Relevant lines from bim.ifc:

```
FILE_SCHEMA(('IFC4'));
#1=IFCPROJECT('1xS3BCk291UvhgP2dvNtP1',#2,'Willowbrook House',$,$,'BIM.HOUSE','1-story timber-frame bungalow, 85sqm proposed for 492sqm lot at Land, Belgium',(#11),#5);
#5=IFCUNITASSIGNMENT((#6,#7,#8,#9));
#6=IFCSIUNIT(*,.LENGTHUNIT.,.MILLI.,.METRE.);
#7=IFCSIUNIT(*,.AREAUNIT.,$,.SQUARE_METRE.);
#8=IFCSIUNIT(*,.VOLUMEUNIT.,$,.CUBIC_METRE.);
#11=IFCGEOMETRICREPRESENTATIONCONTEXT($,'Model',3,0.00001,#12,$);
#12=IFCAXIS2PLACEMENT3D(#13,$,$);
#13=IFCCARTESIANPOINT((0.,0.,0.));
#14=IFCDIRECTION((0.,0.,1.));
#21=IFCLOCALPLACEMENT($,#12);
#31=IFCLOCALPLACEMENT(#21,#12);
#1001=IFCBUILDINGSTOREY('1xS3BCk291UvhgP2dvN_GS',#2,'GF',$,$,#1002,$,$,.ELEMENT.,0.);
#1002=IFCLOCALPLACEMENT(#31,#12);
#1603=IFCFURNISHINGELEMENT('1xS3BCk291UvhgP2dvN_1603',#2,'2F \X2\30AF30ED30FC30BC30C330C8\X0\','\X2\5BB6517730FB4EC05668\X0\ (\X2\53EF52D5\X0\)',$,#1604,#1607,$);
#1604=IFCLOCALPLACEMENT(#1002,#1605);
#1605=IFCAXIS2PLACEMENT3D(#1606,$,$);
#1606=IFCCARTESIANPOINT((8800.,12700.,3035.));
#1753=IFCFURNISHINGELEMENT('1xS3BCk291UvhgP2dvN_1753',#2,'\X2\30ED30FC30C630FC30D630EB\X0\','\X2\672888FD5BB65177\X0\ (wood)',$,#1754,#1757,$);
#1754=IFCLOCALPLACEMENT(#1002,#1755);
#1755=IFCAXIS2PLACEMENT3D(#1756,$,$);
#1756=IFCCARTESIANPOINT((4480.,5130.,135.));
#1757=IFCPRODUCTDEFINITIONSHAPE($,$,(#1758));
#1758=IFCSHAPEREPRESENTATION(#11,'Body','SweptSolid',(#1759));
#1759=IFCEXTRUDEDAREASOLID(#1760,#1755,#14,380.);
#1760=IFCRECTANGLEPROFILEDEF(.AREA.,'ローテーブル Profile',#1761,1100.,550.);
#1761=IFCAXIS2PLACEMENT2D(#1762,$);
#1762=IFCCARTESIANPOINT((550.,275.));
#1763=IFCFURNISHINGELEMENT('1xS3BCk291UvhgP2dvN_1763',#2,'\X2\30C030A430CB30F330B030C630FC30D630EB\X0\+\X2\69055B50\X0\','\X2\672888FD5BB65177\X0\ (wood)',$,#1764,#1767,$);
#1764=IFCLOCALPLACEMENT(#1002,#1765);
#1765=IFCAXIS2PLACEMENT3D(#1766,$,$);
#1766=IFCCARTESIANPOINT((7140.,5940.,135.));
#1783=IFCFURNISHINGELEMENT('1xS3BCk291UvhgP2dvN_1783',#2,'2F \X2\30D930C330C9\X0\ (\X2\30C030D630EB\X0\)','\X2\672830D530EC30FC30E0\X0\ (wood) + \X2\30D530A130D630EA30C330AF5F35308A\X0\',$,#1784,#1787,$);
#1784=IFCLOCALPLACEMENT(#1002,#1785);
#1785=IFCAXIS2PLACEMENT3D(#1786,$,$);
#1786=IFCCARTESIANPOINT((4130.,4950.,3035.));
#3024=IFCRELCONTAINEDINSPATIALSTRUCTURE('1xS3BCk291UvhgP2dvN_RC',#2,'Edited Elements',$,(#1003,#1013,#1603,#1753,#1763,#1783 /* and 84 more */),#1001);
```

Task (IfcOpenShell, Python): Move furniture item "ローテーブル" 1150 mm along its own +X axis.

```python
import ifcopenshell
import ifcopenshell.api.geometry
import ifcopenshell.util.placement
import ifcopenshell.util.unit

model = ifcopenshell.open("bim.ifc")
unit_scale = ifcopenshell.util.unit.calculate_unit_scale(model)

item = model.by_id(1753)
matrix = ifcopenshell.util.placement.get_local_placement(item.ObjectPlacement)
matrix[:3, 3] += matrix[:3, 0] * 1.15 / unit_scale
ifcopenshell.api.geometry.edit_object_placement(model, product=item, matrix=matrix, is_si=False)

print(ifcopenshell.util.placement.get_local_placement(item.ObjectPlacement).round(3) + 0.0)

model.write("bim_updated.ifc")
```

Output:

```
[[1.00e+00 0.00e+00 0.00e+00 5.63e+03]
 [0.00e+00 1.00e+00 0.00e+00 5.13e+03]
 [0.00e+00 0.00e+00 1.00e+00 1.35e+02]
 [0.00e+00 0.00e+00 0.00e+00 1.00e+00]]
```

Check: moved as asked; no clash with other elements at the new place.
